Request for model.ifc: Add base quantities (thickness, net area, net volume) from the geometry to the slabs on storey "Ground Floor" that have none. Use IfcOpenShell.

First a look at what the model holds.

```python
import ifcopenshell
import ifcopenshell.util.element
import ifcopenshell.util.unit

model = ifcopenshell.open("model.ifc")
print(model.schema)
for unit_type in ("LENGTHUNIT", "AREAUNIT", "VOLUMEUNIT"):
    print(unit_type, ifcopenshell.util.unit.calculate_unit_scale(model, unit_type))
storey = next(s for s in model.by_type("IfcBuildingStorey") if s.Name == "Ground Floor")
slabs = [e for e in ifcopenshell.util.element.get_decomposition(storey) if e.is_a("IfcSlab")]
for e in sorted(slabs, key=lambda e: e.id()):
    print(e.id(), e.is_a(), e.Name, list(ifcopenshell.util.element.get_psets(e, qtos_only=True)), sep=" | ")
```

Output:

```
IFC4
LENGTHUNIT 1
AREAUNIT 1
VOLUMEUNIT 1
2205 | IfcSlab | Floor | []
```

```python
import ifcopenshell
import ifcopenshell.api.pset
import ifcopenshell.geom
import ifcopenshell.util.element
import ifcopenshell.util.shape
import ifcopenshell.util.unit

model = ifcopenshell.open("model.ifc")
unit_scale = ifcopenshell.util.unit.calculate_unit_scale(model)
area_scale = ifcopenshell.util.unit.calculate_unit_scale(model, "AREAUNIT")
volume_scale = ifcopenshell.util.unit.calculate_unit_scale(model, "VOLUMEUNIT")
settings = ifcopenshell.geom.settings()

storey = next(s for s in model.by_type("IfcBuildingStorey") if s.Name == "Ground Floor")
slabs = [e for e in ifcopenshell.util.element.get_decomposition(storey) if e.is_a("IfcSlab")]

for e in sorted(slabs, key=lambda e: e.id()):
    if ifcopenshell.util.element.get_psets(e, qtos_only=True, should_inherit=False):
        continue
    # Geometry comes back in metres, in the element's own axes.
    shape = ifcopenshell.geom.create_shape(settings, e)
    values = {
        "Width": ifcopenshell.util.shape.get_z(shape.geometry) / unit_scale,
        "NetArea": ifcopenshell.util.shape.get_footprint_area(shape.geometry) / area_scale,
        "NetVolume": ifcopenshell.util.shape.get_volume(shape.geometry) / volume_scale,
    }
    qto = ifcopenshell.api.pset.add_qto(model, product=e, name="Qto_SlabBaseQuantities")
    ifcopenshell.api.pset.edit_qto(model, qto=qto, properties=values)
    print(e.id(), {k: round(v, 3) for k, v in values.items()})

model.write("model-out.ifc")
```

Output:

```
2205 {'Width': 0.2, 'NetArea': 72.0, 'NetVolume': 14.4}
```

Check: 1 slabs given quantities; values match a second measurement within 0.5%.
